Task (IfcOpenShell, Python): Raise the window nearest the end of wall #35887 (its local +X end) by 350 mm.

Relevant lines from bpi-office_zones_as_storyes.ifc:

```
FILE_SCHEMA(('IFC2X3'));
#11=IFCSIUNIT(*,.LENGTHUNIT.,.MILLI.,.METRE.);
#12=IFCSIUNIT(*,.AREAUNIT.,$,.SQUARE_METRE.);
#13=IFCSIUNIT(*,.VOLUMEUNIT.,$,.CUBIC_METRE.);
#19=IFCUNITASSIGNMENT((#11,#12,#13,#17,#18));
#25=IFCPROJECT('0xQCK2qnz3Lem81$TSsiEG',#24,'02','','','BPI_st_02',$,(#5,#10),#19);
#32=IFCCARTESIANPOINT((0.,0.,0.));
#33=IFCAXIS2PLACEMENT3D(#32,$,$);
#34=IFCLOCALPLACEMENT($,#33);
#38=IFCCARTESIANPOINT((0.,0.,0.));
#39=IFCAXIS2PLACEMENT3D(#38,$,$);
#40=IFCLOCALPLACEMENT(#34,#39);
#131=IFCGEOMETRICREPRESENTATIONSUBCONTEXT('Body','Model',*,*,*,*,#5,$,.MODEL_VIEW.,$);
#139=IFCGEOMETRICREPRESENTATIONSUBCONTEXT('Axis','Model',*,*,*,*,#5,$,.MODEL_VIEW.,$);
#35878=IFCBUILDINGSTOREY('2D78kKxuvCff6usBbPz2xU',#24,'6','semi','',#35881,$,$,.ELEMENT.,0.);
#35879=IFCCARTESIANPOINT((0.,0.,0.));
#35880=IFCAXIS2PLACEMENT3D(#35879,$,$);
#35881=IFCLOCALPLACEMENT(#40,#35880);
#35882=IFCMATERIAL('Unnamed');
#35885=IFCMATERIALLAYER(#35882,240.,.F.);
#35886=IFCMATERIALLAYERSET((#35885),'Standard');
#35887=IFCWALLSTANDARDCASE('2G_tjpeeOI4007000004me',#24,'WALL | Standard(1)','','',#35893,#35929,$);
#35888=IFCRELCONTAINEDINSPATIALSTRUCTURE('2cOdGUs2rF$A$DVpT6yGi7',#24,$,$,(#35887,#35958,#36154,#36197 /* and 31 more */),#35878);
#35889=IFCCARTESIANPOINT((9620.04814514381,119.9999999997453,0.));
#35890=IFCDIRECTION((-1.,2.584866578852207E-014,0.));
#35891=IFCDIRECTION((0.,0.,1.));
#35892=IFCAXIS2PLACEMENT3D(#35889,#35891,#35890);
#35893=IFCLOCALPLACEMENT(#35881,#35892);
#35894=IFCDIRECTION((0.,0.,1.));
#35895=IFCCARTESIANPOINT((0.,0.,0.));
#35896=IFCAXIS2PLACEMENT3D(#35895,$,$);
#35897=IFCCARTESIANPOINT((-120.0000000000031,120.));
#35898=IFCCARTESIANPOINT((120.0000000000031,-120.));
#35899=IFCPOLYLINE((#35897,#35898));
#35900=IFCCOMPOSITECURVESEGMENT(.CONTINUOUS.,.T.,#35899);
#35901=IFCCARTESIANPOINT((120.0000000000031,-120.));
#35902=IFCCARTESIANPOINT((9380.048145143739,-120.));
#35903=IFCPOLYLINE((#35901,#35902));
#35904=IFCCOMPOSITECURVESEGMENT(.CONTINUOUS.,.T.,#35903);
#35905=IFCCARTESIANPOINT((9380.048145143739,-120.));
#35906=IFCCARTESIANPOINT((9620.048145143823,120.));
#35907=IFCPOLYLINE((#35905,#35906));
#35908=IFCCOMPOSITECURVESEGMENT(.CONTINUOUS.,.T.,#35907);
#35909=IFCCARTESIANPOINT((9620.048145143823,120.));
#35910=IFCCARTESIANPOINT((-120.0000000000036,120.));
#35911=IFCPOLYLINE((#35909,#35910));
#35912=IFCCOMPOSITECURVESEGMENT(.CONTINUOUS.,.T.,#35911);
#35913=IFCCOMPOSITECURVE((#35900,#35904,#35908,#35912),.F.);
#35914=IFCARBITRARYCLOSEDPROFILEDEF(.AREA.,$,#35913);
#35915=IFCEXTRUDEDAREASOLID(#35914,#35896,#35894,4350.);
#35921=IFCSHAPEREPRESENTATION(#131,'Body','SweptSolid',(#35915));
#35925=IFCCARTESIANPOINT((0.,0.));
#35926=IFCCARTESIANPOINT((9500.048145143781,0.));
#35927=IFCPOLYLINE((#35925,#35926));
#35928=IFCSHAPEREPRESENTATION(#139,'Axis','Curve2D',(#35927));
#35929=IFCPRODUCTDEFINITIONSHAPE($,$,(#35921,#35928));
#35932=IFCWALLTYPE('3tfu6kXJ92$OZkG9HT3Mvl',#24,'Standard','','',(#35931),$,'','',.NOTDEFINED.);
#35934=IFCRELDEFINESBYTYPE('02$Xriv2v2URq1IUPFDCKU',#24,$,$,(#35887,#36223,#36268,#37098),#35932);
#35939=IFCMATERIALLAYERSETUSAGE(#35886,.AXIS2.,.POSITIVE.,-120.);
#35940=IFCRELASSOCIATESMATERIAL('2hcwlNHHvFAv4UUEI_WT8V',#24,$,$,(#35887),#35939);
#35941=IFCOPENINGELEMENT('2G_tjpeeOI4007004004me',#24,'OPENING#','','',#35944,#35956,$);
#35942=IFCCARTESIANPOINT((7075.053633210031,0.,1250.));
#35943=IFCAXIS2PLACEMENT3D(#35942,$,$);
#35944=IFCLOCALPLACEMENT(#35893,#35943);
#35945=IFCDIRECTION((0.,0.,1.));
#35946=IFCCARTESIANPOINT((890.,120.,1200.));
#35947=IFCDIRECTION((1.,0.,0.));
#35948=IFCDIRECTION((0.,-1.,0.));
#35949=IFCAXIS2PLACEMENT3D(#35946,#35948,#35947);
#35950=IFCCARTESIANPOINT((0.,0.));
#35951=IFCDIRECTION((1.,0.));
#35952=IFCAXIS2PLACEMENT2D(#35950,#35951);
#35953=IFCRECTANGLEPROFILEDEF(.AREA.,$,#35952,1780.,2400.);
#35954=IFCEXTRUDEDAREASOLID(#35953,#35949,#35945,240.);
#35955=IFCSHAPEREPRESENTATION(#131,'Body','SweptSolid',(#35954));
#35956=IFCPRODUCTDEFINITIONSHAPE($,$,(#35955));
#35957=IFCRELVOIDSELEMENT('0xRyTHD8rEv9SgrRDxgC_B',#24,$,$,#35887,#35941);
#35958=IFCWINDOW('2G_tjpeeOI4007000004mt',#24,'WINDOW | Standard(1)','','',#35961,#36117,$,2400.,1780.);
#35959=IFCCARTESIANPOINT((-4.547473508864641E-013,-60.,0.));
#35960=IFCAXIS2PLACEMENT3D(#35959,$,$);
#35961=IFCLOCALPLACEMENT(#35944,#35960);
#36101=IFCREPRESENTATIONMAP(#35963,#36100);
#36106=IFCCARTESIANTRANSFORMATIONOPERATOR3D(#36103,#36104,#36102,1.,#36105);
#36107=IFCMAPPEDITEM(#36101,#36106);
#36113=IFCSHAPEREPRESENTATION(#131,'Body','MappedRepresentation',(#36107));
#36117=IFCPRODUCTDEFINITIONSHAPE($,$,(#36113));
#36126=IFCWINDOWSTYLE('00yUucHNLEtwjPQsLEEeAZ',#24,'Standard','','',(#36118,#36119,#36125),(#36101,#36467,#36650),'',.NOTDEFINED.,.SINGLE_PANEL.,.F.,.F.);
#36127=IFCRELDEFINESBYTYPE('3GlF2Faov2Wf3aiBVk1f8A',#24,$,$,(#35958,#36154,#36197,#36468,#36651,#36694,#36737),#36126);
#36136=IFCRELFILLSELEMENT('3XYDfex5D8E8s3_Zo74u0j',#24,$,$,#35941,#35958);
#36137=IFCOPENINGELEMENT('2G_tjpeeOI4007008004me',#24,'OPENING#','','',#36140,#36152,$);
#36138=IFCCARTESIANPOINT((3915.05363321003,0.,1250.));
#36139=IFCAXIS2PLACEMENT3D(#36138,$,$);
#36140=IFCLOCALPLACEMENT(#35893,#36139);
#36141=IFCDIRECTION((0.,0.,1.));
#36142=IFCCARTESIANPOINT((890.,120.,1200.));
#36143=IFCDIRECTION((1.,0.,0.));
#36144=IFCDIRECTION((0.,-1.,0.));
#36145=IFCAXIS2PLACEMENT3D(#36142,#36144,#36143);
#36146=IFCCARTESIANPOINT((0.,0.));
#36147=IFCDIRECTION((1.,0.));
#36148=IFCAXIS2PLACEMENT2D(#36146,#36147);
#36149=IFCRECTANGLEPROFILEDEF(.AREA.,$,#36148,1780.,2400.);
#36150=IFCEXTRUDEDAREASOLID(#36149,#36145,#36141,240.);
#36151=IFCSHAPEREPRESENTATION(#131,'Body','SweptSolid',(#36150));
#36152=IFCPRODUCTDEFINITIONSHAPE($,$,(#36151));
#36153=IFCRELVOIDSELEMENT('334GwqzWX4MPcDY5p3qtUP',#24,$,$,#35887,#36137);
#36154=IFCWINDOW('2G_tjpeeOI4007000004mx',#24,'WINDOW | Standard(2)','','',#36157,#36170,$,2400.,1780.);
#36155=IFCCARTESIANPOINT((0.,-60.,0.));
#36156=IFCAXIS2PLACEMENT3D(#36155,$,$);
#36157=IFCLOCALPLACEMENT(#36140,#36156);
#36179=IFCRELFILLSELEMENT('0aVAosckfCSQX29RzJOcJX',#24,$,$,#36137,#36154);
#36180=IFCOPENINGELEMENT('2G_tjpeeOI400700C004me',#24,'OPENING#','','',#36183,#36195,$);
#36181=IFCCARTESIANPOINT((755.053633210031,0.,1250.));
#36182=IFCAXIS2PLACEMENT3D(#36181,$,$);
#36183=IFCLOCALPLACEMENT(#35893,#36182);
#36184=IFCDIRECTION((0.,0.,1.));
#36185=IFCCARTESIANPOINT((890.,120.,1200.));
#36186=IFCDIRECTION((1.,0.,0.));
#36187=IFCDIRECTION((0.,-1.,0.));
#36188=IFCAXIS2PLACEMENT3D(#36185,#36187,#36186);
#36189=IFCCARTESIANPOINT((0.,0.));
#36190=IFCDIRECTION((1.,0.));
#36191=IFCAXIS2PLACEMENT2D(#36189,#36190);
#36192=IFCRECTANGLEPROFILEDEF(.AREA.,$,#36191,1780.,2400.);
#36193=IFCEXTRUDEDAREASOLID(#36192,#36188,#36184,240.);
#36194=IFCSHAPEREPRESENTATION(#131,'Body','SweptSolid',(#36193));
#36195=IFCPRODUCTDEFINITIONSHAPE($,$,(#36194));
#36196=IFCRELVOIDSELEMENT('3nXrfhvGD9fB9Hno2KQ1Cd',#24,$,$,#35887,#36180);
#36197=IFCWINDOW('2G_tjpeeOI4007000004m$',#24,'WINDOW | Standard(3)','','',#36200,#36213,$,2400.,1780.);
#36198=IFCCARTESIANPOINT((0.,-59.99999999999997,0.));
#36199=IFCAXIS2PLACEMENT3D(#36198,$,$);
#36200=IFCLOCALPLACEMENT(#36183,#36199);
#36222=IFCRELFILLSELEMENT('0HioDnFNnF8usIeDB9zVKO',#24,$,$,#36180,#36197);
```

```python
import numpy as np
import ifcopenshell
import ifcopenshell.api.geometry
import ifcopenshell.util.placement
import ifcopenshell.util.unit

model = ifcopenshell.open("bpi-office_zones_as_storyes.ifc")
unit_scale = ifcopenshell.util.unit.calculate_unit_scale(model)

window = model.by_guid("2G_tjpeeOI4007000004mt")
opening = window.FillsVoids[0].RelatingOpeningElement
dz = 350.0

shift = np.array([0.0, 0.0, dz])
# The window is placed relative to its opening, so it follows when the opening moves.
matrix = ifcopenshell.util.placement.get_local_placement(opening.ObjectPlacement)
matrix[:3, 3] += shift
ifcopenshell.api.geometry.edit_object_placement(
    model, product=opening, matrix=matrix, is_si=False, should_transform_children=True
)

print(f"moved by {dz * unit_scale:+.3f} m")

model.write("bpi-office_zones_as_storyes_v2.ifc")
```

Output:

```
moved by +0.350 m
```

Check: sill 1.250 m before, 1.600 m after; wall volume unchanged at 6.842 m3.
